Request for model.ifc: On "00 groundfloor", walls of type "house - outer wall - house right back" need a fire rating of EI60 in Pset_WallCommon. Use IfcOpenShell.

First a look at what the model holds.

```python
import ifcopenshell
import ifcopenshell.util.element

model = ifcopenshell.open("model.ifc")
print(model.schema)
storey = next(s for s in model.by_type("IfcBuildingStorey") if s.Name == "00 groundfloor")
walls = [e for e in ifcopenshell.util.element.get_decomposition(storey) if e.is_a("IfcWall")]
seen = {}
for e in walls:
    element_type = ifcopenshell.util.element.get_type(e)
    key = (element_type.Name if element_type != e and element_type else None, ifcopenshell.util.element.get_pset(e, "Pset_WallCommon", "FireRating"))
    seen[key] = seen.get(key, 0) + 1
for (name, value), count in sorted(seen.items(), key=str):
    print(count, "x", name, "|", value)
```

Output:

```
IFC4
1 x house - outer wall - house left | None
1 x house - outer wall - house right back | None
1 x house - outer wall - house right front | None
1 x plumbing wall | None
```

```python
import ifcopenshell
import ifcopenshell.api.pset
import ifcopenshell.util.element

model = ifcopenshell.open("model.ifc")

storey = next(s for s in model.by_type("IfcBuildingStorey") if s.Name == "00 groundfloor")
walls = [e for e in ifcopenshell.util.element.get_decomposition(storey) if e.is_a("IfcWall")]

count = 0
for e in walls:
    element_type = ifcopenshell.util.element.get_type(e)
    if element_type in (None, e) or element_type.Name != "house - outer wall - house right back":
        continue
    # add_pset returns the element's existing set when there is one.
    pset = ifcopenshell.api.pset.add_pset(model, product=e, name="Pset_WallCommon")
    ifcopenshell.api.pset.edit_pset(model, pset=pset, properties={"FireRating": "EI60"})
    count += 1

print(count, "walls updated")

model.write("model_edited.ifc")
```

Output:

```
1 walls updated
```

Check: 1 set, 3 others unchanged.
